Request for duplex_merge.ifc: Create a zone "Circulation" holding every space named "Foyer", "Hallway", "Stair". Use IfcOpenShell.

First a look at what the model holds.

```python
import ifcopenshell

model = ifcopenshell.open("duplex_merge.ifc")
print(model.schema)
seen = {}
for space in model.by_type("IfcSpace"):
    seen[space.LongName] = seen.get(space.LongName, 0) + 1
for name, count in sorted(seen.items(), key=str):
    print(count, "x", name)
print("zones:", [z.Name for z in model.by_type("IfcZone")][:20])
```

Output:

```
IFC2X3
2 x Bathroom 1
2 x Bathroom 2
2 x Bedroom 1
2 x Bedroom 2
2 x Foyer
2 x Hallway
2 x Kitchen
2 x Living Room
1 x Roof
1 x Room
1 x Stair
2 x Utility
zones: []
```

```python
import ifcopenshell
import ifcopenshell.api.group
import ifcopenshell.api.root

model = ifcopenshell.open("duplex_merge.ifc")

names = {"Foyer", "Hallway", "Stair"}
spaces = [s for s in model.by_type("IfcSpace") if s.LongName in names]

zone = ifcopenshell.api.root.create_entity(model, ifc_class="IfcZone", name="Circulation")
ifcopenshell.api.group.assign_group(model, products=spaces, group=zone)
print(len(spaces), "spaces in", zone.Name)

model.write("duplex_merge_rev.ifc")
```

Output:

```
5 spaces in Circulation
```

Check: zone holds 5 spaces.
